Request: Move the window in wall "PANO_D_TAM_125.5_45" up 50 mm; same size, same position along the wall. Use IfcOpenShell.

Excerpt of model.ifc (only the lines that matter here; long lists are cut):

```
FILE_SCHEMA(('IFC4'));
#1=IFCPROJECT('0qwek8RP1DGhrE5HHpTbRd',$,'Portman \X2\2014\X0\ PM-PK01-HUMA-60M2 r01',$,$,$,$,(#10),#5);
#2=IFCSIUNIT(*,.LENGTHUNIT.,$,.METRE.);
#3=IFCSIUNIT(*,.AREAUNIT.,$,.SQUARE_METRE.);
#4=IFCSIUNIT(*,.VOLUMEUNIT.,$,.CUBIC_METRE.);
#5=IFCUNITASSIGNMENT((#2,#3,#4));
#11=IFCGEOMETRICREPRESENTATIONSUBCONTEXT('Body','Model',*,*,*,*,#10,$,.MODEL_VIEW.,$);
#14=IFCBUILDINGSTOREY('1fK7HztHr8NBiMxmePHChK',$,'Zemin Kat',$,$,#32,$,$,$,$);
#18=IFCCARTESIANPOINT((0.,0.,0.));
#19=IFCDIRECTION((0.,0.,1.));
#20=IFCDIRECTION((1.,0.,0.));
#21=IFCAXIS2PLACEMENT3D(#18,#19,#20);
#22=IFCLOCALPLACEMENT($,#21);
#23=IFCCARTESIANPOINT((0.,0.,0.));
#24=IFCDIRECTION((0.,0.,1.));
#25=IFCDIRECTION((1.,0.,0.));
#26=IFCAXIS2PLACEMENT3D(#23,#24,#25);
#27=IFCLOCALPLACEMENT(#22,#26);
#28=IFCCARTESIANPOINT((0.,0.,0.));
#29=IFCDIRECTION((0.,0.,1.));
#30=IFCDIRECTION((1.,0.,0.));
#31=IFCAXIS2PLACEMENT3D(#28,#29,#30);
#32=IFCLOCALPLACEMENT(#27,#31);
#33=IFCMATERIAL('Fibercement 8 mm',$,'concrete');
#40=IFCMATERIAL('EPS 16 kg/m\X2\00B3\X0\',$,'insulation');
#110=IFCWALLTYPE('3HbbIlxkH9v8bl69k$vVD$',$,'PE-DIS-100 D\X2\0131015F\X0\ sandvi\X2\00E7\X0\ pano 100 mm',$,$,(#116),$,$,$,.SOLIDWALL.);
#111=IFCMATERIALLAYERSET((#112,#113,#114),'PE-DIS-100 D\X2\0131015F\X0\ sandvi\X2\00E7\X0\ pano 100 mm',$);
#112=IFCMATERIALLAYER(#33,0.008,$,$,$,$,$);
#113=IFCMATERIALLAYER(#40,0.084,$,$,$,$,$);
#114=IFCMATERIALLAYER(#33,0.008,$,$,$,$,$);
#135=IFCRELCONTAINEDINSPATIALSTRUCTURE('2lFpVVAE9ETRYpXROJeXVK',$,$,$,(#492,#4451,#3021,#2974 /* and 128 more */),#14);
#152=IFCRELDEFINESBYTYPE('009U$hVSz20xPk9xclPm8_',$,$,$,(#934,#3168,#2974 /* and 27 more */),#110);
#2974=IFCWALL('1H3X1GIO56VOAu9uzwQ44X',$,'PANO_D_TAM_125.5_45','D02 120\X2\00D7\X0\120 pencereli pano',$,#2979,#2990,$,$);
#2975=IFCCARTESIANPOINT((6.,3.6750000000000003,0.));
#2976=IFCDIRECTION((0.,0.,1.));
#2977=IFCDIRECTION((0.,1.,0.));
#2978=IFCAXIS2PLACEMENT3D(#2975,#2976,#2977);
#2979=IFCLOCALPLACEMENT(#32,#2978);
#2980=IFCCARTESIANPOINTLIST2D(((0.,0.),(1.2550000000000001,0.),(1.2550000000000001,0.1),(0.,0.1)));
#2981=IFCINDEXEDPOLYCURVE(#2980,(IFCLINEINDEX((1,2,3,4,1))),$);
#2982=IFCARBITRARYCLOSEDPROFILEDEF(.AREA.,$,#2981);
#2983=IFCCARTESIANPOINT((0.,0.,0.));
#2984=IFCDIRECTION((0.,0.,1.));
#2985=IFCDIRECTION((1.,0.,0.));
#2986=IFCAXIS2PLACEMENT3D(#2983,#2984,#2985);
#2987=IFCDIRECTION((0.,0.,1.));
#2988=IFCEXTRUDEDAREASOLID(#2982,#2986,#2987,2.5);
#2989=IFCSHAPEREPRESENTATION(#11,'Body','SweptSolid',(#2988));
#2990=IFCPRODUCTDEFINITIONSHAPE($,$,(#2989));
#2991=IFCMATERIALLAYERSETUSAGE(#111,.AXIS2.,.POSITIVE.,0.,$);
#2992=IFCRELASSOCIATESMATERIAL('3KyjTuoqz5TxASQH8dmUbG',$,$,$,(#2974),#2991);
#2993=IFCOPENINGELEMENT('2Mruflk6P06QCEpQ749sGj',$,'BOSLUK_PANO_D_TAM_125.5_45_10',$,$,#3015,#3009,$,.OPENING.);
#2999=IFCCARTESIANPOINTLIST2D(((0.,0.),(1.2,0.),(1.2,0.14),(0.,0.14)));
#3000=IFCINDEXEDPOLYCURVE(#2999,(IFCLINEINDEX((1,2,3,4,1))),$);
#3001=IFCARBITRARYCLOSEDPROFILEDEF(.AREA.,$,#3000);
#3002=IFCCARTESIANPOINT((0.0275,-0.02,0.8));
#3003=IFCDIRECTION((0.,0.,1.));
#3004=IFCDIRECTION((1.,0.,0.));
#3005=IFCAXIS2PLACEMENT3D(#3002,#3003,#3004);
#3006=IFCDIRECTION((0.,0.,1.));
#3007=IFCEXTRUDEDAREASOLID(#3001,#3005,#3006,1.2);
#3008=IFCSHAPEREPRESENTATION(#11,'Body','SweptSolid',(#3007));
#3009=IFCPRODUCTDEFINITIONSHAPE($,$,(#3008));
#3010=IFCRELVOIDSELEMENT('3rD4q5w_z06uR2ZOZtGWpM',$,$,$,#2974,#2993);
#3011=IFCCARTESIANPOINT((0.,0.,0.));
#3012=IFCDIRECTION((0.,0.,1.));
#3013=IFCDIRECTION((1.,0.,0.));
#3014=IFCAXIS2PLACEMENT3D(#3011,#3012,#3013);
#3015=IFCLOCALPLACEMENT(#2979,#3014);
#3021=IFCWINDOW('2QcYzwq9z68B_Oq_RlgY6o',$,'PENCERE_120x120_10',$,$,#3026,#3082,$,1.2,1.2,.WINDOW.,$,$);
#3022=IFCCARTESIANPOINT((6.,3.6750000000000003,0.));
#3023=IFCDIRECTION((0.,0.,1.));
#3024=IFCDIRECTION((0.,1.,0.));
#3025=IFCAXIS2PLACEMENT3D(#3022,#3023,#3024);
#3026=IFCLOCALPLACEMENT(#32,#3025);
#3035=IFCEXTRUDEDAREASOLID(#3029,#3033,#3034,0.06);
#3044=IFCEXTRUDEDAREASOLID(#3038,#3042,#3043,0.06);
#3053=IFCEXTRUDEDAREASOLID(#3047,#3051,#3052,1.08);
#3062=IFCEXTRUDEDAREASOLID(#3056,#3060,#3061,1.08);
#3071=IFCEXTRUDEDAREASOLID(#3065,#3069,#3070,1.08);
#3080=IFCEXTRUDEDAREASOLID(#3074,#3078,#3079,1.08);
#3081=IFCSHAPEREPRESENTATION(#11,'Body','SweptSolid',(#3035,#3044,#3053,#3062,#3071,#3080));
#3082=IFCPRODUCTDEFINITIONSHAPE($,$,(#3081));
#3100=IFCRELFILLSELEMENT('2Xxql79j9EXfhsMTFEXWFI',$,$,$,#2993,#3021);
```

```python
import numpy as np
import ifcopenshell
import ifcopenshell.api.geometry
import ifcopenshell.util.placement
import ifcopenshell.util.unit

model = ifcopenshell.open("model.ifc")
unit_scale = ifcopenshell.util.unit.calculate_unit_scale(model)

window = model.by_id(3021)
opening = window.FillsVoids[0].RelatingOpeningElement
dz = 0.05 / unit_scale

shift = np.array([0.0, 0.0, dz])
# The window is not placed relative to its opening, so move both.
for product in (opening, window):
    matrix = ifcopenshell.util.placement.get_local_placement(product.ObjectPlacement)
    matrix[:3, 3] += shift
    ifcopenshell.api.geometry.edit_object_placement(model, product=product, matrix=matrix, is_si=False)

print(f"moved by {dz * unit_scale:+.3f} m")

model.write("model-out.ifc")
```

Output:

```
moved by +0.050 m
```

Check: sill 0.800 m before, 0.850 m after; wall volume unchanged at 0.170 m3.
